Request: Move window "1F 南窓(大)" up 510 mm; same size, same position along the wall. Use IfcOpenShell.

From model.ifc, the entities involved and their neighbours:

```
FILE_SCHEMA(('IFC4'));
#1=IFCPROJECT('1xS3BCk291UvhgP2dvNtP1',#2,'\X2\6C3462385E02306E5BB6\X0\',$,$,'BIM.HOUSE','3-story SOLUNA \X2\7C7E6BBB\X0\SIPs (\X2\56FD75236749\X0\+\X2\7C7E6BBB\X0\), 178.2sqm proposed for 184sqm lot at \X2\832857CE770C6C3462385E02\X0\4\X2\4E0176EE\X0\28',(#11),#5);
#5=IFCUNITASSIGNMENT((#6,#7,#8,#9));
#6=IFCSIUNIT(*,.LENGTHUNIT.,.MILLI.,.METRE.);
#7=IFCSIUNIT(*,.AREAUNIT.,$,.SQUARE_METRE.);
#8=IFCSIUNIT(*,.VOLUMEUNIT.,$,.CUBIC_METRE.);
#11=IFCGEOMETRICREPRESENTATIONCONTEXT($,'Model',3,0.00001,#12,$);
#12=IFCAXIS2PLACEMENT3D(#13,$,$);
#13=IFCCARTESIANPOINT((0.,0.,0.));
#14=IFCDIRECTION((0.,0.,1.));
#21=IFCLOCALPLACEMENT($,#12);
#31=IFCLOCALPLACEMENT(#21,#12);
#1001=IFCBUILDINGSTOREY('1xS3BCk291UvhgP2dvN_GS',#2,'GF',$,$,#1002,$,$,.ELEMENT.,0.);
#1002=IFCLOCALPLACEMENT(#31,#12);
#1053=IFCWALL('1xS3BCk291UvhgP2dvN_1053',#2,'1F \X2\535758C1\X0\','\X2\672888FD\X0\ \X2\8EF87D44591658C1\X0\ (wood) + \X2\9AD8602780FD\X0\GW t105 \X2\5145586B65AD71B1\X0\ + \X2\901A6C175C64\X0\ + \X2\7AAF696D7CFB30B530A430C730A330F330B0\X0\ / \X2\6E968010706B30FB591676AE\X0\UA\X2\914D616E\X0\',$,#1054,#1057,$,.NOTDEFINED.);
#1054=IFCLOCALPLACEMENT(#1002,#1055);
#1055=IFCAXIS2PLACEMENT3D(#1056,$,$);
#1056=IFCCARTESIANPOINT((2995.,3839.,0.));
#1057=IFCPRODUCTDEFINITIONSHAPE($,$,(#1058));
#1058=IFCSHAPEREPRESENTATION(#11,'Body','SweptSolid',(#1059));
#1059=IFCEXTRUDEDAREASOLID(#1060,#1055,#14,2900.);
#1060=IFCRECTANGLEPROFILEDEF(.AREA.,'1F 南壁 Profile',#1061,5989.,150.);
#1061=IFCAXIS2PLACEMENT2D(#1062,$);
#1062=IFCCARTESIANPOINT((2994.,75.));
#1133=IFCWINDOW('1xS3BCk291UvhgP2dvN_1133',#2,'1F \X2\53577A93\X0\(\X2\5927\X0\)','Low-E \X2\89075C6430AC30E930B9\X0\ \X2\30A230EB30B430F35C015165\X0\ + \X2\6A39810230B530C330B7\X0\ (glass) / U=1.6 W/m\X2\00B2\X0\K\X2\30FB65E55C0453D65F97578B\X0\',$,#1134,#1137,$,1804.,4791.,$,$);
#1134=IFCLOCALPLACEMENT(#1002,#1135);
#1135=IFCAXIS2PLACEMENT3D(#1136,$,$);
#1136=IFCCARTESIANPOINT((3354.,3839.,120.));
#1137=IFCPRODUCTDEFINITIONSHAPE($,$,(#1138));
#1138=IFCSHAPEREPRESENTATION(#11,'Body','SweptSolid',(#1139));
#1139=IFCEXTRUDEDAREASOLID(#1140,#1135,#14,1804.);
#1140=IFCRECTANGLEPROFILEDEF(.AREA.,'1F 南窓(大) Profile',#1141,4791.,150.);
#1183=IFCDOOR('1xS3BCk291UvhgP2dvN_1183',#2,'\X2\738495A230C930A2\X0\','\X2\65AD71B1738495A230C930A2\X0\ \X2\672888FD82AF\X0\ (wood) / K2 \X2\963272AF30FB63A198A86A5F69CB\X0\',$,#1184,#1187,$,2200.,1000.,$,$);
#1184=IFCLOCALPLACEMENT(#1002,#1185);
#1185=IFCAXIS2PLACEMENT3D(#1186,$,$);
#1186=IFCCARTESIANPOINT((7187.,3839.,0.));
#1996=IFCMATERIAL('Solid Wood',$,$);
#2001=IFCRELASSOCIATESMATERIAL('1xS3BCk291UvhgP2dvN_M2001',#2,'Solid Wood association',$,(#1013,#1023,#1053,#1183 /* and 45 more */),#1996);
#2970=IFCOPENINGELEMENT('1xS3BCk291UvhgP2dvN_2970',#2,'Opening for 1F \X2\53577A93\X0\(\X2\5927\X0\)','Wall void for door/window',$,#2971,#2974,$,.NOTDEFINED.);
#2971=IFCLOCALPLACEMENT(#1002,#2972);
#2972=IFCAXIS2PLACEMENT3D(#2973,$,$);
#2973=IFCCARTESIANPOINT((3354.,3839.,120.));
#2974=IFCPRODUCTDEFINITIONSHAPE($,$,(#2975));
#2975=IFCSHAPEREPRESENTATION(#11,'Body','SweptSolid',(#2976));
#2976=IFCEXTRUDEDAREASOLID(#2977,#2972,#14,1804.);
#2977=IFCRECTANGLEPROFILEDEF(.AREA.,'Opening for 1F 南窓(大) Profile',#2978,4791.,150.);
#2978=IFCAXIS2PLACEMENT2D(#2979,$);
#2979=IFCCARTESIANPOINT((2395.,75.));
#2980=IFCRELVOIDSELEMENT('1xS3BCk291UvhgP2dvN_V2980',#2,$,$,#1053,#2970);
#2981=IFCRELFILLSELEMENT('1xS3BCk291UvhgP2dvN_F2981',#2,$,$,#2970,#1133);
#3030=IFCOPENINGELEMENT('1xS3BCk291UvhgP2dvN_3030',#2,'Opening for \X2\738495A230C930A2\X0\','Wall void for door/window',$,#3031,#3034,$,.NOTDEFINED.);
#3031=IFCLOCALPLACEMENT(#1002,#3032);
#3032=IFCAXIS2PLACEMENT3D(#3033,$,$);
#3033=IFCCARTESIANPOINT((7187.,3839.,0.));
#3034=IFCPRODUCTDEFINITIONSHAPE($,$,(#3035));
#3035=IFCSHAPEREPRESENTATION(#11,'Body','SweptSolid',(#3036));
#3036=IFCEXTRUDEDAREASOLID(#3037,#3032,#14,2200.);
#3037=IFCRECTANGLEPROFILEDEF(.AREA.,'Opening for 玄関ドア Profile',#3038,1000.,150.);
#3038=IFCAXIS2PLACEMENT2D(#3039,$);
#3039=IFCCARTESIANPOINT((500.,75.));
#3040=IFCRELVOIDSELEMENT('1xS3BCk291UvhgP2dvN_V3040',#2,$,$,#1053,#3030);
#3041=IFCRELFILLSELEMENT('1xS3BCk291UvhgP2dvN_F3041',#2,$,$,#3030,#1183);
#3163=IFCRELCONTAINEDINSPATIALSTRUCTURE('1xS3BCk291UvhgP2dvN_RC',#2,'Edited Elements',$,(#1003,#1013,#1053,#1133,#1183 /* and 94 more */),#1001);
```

```python
import numpy as np
import ifcopenshell
import ifcopenshell.api.geometry
import ifcopenshell.util.placement
import ifcopenshell.util.unit

model = ifcopenshell.open("model.ifc")
unit_scale = ifcopenshell.util.unit.calculate_unit_scale(model)

window = model.by_guid("1xS3BCk291UvhgP2dvN_1133")
opening = window.FillsVoids[0].RelatingOpeningElement
dz = 510.0

shift = np.array([0.0, 0.0, dz])
# The window is not placed relative to its opening, so move both.
for product in (opening, window):
    matrix = ifcopenshell.util.placement.get_local_placement(product.ObjectPlacement)
    matrix[:3, 3] += shift
    ifcopenshell.api.geometry.edit_object_placement(model, product=product, matrix=matrix, is_si=False)

print(f"moved by {dz * unit_scale:+.3f} m")

model.write("model_updated.ifc")
```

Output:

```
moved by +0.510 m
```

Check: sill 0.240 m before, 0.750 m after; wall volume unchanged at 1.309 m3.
